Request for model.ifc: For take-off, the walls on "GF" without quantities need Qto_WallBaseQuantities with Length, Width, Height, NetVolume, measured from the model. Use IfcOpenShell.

First a look at what the model holds.

```python
import ifcopenshell
import ifcopenshell.util.element
import ifcopenshell.util.unit

model = ifcopenshell.open("model.ifc")
print(model.schema)
for unit_type in ("LENGTHUNIT", "AREAUNIT", "VOLUMEUNIT"):
    print(unit_type, ifcopenshell.util.unit.calculate_unit_scale(model, unit_type))
storey = next(s for s in model.by_type("IfcBuildingStorey") if s.Name == "GF")
walls = [e for e in ifcopenshell.util.element.get_decomposition(storey) if e.is_a("IfcWall")]
for e in sorted(walls, key=lambda e: e.id()):
    print(e.id(), e.is_a(), e.Name, list(ifcopenshell.util.element.get_psets(e, qtos_only=True)), sep=" | ")
```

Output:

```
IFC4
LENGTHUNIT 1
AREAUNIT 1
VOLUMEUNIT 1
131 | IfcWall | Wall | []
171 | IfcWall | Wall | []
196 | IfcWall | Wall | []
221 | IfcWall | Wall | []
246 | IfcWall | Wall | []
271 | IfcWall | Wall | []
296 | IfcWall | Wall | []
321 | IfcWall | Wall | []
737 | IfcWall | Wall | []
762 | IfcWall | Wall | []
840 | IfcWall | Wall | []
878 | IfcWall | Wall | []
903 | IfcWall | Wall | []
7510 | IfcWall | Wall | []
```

```python
import ifcopenshell
import ifcopenshell.api.pset
import ifcopenshell.geom
import ifcopenshell.util.element
import ifcopenshell.util.shape
import ifcopenshell.util.unit

model = ifcopenshell.open("model.ifc")
unit_scale = ifcopenshell.util.unit.calculate_unit_scale(model)
volume_scale = ifcopenshell.util.unit.calculate_unit_scale(model, "VOLUMEUNIT")
settings = ifcopenshell.geom.settings()

storey = next(s for s in model.by_type("IfcBuildingStorey") if s.Name == "GF")
walls = [e for e in ifcopenshell.util.element.get_decomposition(storey) if e.is_a("IfcWall")]

for e in sorted(walls, key=lambda e: e.id()):
    if ifcopenshell.util.element.get_psets(e, qtos_only=True, should_inherit=False):
        continue
    # Geometry comes back in metres, in the element's own axes.
    shape = ifcopenshell.geom.create_shape(settings, e)
    values = {
        "Length": ifcopenshell.util.shape.get_x(shape.geometry) / unit_scale,
        "Width": ifcopenshell.util.shape.get_y(shape.geometry) / unit_scale,
        "Height": ifcopenshell.util.shape.get_z(shape.geometry) / unit_scale,
        "NetVolume": ifcopenshell.util.shape.get_volume(shape.geometry) / volume_scale,
    }
    qto = ifcopenshell.api.pset.add_qto(model, product=e, name="Qto_WallBaseQuantities")
    ifcopenshell.api.pset.edit_qto(model, qto=qto, properties=values)
    print(e.id(), {k: round(v, 3) for k, v in values.items()})

model.write("model_v2.ifc")
```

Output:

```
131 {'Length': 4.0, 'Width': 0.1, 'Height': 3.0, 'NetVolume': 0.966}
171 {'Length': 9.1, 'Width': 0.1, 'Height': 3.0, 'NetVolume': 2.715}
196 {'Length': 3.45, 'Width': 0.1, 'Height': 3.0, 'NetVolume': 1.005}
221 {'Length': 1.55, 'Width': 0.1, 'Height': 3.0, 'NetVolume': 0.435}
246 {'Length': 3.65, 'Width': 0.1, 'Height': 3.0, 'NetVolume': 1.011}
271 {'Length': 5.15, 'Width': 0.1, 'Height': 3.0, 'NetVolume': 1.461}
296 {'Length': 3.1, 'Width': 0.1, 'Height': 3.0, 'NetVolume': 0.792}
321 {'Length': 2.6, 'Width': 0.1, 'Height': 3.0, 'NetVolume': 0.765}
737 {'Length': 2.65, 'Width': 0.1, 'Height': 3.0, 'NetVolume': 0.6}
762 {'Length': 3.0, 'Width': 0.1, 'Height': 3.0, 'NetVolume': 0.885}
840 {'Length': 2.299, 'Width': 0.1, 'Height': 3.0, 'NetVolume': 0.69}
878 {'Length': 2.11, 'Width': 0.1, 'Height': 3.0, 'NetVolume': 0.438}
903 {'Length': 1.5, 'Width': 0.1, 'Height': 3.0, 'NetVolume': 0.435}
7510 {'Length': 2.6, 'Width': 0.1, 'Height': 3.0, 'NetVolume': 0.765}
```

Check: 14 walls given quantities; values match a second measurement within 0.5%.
